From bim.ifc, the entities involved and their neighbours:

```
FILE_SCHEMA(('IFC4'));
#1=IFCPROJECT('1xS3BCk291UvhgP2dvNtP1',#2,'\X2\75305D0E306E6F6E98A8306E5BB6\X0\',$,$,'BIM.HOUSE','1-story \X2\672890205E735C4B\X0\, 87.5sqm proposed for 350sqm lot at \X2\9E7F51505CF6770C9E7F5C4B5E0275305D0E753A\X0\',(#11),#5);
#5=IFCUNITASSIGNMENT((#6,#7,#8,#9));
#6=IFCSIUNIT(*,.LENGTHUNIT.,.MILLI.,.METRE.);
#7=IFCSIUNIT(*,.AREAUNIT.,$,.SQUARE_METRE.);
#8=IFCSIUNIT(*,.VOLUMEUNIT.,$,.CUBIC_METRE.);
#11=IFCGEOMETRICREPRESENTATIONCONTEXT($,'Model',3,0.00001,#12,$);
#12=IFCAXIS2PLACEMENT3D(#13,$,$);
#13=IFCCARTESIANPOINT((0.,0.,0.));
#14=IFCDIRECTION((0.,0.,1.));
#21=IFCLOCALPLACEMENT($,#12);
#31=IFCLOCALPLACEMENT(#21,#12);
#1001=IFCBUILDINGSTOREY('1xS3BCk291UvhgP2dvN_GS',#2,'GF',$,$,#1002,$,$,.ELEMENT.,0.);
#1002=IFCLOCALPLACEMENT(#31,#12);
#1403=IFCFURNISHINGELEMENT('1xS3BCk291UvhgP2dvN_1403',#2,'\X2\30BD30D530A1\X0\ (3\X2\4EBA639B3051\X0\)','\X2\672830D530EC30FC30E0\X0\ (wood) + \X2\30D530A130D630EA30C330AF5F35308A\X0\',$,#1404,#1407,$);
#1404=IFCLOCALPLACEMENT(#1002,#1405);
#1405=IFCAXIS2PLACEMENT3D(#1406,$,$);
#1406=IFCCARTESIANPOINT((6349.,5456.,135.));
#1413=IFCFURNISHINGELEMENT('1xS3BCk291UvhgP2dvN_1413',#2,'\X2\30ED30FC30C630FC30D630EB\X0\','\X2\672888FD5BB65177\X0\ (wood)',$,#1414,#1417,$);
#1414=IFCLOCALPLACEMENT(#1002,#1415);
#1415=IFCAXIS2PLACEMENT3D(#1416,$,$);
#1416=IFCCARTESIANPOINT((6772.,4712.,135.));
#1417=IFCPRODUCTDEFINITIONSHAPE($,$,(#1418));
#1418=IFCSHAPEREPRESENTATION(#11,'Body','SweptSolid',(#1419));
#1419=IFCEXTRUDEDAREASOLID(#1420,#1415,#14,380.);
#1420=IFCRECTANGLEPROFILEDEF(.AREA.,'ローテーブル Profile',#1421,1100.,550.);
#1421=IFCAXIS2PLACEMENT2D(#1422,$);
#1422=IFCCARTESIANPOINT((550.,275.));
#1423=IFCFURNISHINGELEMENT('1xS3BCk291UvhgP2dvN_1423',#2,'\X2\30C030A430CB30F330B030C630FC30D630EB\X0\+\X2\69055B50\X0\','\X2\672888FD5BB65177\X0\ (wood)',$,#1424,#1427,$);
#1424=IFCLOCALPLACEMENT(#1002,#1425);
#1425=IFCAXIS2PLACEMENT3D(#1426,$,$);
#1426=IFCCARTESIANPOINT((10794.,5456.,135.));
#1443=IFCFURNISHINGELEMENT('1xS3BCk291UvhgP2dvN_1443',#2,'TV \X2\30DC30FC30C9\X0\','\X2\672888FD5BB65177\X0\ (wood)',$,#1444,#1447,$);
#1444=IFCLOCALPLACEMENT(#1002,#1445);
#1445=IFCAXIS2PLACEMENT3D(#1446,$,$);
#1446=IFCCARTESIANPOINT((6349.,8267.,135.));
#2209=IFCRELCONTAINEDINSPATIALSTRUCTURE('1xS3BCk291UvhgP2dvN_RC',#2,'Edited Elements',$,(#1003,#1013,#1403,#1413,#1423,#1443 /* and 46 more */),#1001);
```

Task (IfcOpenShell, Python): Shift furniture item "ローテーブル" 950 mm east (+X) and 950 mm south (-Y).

```python
import ifcopenshell
import ifcopenshell.api.geometry
import ifcopenshell.util.placement
import ifcopenshell.util.unit

model = ifcopenshell.open("bim.ifc")
unit_scale = ifcopenshell.util.unit.calculate_unit_scale(model)

item = model.by_guid("1xS3BCk291UvhgP2dvN_1413")
matrix = ifcopenshell.util.placement.get_local_placement(item.ObjectPlacement)
matrix[0, 3] += 0.95 / unit_scale
matrix[1, 3] -= 0.95 / unit_scale
ifcopenshell.api.geometry.edit_object_placement(model, product=item, matrix=matrix, is_si=False)

print(ifcopenshell.util.placement.get_local_placement(item.ObjectPlacement).round(3) + 0.0)

model.write("bim_rev.ifc")
```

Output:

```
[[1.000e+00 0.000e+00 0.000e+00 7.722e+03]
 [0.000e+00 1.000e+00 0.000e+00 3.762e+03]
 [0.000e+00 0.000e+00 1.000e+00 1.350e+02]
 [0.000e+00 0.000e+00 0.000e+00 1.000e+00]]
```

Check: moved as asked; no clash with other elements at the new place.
